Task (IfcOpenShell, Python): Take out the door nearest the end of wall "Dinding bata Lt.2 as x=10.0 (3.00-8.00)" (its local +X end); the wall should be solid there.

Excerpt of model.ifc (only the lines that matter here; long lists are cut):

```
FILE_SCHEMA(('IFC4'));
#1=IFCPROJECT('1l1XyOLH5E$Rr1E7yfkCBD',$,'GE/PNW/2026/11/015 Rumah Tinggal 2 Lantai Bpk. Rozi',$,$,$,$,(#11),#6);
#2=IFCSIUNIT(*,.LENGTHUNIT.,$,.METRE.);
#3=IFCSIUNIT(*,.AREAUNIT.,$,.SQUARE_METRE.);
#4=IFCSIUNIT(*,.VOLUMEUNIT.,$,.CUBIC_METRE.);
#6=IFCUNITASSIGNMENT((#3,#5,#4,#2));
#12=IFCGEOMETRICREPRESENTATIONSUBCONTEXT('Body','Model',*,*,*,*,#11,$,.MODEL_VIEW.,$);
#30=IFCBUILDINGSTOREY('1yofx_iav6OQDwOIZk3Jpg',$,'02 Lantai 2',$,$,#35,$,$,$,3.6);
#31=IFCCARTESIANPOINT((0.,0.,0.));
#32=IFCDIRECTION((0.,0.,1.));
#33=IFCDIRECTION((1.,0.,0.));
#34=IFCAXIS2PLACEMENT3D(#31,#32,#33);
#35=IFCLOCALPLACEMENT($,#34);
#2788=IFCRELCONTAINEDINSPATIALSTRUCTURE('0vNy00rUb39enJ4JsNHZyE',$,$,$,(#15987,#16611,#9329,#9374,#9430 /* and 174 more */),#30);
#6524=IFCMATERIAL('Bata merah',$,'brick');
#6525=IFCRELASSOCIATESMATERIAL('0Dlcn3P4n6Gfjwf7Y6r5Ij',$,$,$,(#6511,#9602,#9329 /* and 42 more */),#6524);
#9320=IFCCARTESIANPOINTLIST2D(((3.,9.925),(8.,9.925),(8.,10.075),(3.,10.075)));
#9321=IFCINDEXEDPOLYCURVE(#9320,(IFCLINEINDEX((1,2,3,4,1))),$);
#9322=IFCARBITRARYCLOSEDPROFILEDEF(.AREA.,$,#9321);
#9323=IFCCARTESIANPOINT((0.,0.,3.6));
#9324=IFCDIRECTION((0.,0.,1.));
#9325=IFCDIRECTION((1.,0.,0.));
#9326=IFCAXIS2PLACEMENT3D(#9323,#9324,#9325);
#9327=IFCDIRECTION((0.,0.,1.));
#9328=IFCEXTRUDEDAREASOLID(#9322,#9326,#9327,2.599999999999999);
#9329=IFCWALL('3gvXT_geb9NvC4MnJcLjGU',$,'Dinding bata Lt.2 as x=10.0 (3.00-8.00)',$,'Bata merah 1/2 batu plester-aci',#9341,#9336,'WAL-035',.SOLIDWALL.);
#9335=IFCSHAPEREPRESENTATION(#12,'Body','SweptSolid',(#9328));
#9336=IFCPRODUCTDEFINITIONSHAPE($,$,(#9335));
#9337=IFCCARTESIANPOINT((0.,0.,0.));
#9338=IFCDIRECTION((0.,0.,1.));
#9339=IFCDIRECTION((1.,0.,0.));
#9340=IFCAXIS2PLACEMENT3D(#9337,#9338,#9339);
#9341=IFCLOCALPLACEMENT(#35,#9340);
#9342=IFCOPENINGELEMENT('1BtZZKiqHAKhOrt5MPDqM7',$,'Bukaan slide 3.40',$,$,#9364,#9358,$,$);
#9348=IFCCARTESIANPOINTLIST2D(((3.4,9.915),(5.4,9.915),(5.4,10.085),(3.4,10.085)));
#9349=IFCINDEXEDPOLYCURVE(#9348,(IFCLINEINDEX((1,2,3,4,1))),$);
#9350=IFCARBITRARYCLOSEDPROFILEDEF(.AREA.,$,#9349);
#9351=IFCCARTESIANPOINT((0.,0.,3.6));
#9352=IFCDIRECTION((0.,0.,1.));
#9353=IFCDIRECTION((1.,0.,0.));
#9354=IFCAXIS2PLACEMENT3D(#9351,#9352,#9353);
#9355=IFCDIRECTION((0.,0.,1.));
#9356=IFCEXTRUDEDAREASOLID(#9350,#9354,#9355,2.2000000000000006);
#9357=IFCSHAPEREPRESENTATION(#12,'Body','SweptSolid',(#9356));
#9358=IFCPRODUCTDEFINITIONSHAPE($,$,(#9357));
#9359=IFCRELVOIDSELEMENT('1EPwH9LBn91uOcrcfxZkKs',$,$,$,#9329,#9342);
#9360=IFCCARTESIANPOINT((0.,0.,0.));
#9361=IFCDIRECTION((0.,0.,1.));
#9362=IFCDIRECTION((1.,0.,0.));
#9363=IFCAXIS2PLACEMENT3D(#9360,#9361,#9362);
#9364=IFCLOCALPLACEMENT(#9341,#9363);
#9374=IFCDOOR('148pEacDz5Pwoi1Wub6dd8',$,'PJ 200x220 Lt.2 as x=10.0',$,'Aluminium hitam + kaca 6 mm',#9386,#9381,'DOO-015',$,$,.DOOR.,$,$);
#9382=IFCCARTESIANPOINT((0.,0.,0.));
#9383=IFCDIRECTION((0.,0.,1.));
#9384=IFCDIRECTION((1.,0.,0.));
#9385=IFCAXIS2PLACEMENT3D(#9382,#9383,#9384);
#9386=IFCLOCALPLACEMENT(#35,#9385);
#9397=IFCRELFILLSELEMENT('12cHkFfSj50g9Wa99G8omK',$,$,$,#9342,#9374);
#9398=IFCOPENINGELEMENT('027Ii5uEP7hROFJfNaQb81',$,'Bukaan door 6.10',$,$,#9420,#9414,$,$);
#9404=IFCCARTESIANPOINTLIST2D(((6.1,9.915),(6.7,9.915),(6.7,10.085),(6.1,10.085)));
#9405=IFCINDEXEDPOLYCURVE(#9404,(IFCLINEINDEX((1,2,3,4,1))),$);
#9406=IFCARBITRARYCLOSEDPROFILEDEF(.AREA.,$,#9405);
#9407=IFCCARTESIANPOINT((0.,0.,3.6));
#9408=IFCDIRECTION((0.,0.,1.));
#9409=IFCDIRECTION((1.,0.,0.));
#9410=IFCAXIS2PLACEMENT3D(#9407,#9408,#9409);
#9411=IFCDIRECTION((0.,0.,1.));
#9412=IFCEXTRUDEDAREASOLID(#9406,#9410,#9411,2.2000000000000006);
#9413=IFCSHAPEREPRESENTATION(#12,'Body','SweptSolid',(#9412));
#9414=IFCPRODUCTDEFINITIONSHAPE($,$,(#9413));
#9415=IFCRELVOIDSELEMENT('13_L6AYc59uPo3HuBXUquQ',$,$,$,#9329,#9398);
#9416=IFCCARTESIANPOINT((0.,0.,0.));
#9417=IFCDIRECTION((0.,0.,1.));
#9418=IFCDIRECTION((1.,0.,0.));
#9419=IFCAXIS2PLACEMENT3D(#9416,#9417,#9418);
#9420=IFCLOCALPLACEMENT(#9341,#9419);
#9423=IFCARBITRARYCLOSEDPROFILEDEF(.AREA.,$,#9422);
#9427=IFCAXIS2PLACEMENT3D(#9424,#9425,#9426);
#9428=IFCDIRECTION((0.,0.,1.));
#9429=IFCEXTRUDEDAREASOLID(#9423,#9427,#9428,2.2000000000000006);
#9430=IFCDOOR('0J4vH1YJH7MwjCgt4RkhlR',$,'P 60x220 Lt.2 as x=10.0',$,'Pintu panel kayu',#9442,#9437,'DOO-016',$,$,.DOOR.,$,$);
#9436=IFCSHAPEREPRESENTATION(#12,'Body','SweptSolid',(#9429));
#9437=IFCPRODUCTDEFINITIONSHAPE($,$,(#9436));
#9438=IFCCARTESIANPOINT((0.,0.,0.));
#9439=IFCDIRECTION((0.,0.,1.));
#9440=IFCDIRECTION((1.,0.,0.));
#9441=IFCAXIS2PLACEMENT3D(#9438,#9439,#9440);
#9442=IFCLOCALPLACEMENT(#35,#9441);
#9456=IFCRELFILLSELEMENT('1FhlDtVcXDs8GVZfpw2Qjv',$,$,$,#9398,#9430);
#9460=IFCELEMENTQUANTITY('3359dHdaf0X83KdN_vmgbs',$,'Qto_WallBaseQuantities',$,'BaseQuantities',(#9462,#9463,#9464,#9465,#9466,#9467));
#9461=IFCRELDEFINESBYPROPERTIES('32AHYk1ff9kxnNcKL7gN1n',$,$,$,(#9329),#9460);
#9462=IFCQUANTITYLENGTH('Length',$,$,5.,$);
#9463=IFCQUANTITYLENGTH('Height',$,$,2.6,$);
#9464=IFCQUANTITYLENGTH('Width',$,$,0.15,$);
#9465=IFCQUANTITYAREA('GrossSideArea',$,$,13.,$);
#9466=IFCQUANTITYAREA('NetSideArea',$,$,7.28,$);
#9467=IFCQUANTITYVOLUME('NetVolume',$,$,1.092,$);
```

```python
import ifcopenshell
import ifcopenshell.api.feature
import ifcopenshell.api.pset
import ifcopenshell.api.root
import ifcopenshell.geom
import ifcopenshell.util.element
import ifcopenshell.util.shape
import ifcopenshell.util.unit

model = ifcopenshell.open("model.ifc")
area_scale = ifcopenshell.util.unit.calculate_unit_scale(model, "AREAUNIT")
volume_scale = ifcopenshell.util.unit.calculate_unit_scale(model, "VOLUMEUNIT")
settings = ifcopenshell.geom.settings()


def volume(element):
    """Net volume in cubic metres, openings subtracted."""
    shape = ifcopenshell.geom.create_shape(settings, element)
    return ifcopenshell.util.shape.get_volume(shape.geometry)


door = model.by_guid("0J4vH1YJH7MwjCgt4RkhlR")
opening = door.FillsVoids[0].RelatingOpeningElement
wall = opening.VoidsElements[0].RelatingBuildingElement
before = volume(wall)

ifcopenshell.api.root.remove_product(model, product=door)
ifcopenshell.api.feature.remove_feature(model, feature=opening)

after = volume(wall)
thickness = 0.15  # wall thickness in metres

# Update the wall's stored quantities.
qto = model.by_id(ifcopenshell.util.element.get_pset(wall, "Qto_WallBaseQuantities", should_inherit=False)["id"])
ifcopenshell.api.pset.edit_qto(model, qto=qto, properties={
    "NetSideArea": after / thickness / area_scale,
    "NetVolume": after / volume_scale,
})

print(f"wall volume {before:.3f} -> {after:.3f} m3")

model.write("model_updated.ifc")
```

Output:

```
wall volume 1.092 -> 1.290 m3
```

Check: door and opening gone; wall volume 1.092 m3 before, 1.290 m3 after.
